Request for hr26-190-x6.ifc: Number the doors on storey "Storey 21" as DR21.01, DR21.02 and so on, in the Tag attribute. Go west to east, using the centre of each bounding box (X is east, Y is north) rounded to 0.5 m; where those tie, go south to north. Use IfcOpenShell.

First a look at what the model holds.

```python
import ifcopenshell
import ifcopenshell.util.element
import ifcopenshell.util.placement

model = ifcopenshell.open("hr26-190-x6.ifc")
print(model.schema)
storey = next(s for s in model.by_type("IfcBuildingStorey") if s.Name == "Storey 21")
doors = [e for e in ifcopenshell.util.element.get_decomposition(storey) if e.is_a("IfcDoor")]
for e in sorted(doors, key=lambda e: e.id()):
    origin = ifcopenshell.util.placement.get_local_placement(e.ObjectPlacement)[:3, 3]
    print(e.id(), e.Tag, e.Name, origin.round(2) + 0.0, sep=" | ")
```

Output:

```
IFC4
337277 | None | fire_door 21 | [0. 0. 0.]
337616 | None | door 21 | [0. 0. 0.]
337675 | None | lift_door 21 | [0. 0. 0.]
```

```python
import ifcopenshell
import ifcopenshell.geom
import ifcopenshell.util.element
import ifcopenshell.util.shape

model = ifcopenshell.open("hr26-190-x6.ifc")
settings = ifcopenshell.geom.settings()
settings.set("use-world-coords", True)


def centre(element):
    shape = ifcopenshell.geom.create_shape(settings, element)
    return ifcopenshell.util.shape.get_bbox_centroid(shape.geometry)


storey = next(s for s in model.by_type("IfcBuildingStorey") if s.Name == "Storey 21")
doors = [e for e in ifcopenshell.util.element.get_decomposition(storey) if e.is_a("IfcDoor")]

# Insertion points can sit at a corner or the storey origin, so sort by the geometry (in metres).
centres = {e: centre(e) for e in doors}
doors.sort(key=lambda e: (round(centres[e][0] / 0.5), centres[e][1]))

for i, e in enumerate(doors, start=1):
    number = f"DR21.{i:02d}"
    e.Tag = number
    print(e.id(), number)

model.write("hr26-190-x6_v2.ifc")
```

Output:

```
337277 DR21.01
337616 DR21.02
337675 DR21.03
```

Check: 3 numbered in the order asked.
